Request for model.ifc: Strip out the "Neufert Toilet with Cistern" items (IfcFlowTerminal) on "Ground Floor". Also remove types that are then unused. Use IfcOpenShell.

First a look at what the model holds.

```python
import ifcopenshell
import ifcopenshell.util.element

model = ifcopenshell.open("model.ifc")
print(model.schema)
storey = next(s for s in model.by_type("IfcBuildingStorey") if s.Name == "Ground Floor")
terminals = [e for e in ifcopenshell.util.element.get_decomposition(storey) if e.is_a("IfcFlowTerminal")]
seen = {}
for e in terminals:
    element_type = ifcopenshell.util.element.get_type(e)
    name = element_type.Name if element_type not in (None, e) else None
    seen[name] = seen.get(name, 0) + 1
for name, count in sorted(seen.items(), key=str):
    print(count, "x", name)
```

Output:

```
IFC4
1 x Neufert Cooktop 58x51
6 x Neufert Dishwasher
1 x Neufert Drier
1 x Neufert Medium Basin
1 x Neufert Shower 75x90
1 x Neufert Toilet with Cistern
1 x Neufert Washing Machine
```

```python
import ifcopenshell
import ifcopenshell.api.root
import ifcopenshell.util.element

model = ifcopenshell.open("model.ifc")

storey = next(s for s in model.by_type("IfcBuildingStorey") if s.Name == "Ground Floor")
terminals = [e for e in ifcopenshell.util.element.get_decomposition(storey) if e.is_a("IfcFlowTerminal")]
targets = [e for e in terminals if (t := ifcopenshell.util.element.get_type(e)) not in (None, e) and t.Name == "Neufert Toilet with Cistern"]
types = {ifcopenshell.util.element.get_type(e) for e in targets} - {None, *targets}

for e in targets:
    ifcopenshell.api.root.remove_product(model, product=e)
print(len(targets), "removed")

unused = [t for t in types if not ifcopenshell.util.element.get_types(t)]
for t in unused:
    ifcopenshell.api.root.remove_product(model, product=t)
print(len(unused), "unused types removed")

model.write("model_edited.ifc")
```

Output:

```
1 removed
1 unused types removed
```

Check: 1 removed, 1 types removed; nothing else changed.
